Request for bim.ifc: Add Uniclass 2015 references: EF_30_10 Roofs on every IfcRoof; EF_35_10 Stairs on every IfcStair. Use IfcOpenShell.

First a look at what the model holds.

```python
import ifcopenshell

model = ifcopenshell.open("bim.ifc")
print(model.schema)
print("classifications:", [c.Name for c in model.by_type("IfcClassification")])
for ifc_class in ("IfcDoor", "IfcRoof", "IfcStair", "IfcWall", "IfcWindow"):
    print(ifc_class, len(model.by_type(ifc_class)))
```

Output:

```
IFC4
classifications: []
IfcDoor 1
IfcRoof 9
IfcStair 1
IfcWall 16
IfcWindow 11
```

```python
import ifcopenshell
import ifcopenshell.api.classification

model = ifcopenshell.open("bim.ifc")

system = ifcopenshell.api.classification.add_classification(model, classification="Uniclass 2015")

codes = {
    "IfcRoof": ("EF_30_10", "Roofs"),
    "IfcStair": ("EF_35_10", "Stairs"),
}
for ifc_class, (code, name) in codes.items():
    products = model.by_type(ifc_class)
    ifcopenshell.api.classification.add_reference(
        model, products=products, classification=system, identification=code, name=name
    )
    print(code, len(products))

model.write("bim_v2.ifc")
```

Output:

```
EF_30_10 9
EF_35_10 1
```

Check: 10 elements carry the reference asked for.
